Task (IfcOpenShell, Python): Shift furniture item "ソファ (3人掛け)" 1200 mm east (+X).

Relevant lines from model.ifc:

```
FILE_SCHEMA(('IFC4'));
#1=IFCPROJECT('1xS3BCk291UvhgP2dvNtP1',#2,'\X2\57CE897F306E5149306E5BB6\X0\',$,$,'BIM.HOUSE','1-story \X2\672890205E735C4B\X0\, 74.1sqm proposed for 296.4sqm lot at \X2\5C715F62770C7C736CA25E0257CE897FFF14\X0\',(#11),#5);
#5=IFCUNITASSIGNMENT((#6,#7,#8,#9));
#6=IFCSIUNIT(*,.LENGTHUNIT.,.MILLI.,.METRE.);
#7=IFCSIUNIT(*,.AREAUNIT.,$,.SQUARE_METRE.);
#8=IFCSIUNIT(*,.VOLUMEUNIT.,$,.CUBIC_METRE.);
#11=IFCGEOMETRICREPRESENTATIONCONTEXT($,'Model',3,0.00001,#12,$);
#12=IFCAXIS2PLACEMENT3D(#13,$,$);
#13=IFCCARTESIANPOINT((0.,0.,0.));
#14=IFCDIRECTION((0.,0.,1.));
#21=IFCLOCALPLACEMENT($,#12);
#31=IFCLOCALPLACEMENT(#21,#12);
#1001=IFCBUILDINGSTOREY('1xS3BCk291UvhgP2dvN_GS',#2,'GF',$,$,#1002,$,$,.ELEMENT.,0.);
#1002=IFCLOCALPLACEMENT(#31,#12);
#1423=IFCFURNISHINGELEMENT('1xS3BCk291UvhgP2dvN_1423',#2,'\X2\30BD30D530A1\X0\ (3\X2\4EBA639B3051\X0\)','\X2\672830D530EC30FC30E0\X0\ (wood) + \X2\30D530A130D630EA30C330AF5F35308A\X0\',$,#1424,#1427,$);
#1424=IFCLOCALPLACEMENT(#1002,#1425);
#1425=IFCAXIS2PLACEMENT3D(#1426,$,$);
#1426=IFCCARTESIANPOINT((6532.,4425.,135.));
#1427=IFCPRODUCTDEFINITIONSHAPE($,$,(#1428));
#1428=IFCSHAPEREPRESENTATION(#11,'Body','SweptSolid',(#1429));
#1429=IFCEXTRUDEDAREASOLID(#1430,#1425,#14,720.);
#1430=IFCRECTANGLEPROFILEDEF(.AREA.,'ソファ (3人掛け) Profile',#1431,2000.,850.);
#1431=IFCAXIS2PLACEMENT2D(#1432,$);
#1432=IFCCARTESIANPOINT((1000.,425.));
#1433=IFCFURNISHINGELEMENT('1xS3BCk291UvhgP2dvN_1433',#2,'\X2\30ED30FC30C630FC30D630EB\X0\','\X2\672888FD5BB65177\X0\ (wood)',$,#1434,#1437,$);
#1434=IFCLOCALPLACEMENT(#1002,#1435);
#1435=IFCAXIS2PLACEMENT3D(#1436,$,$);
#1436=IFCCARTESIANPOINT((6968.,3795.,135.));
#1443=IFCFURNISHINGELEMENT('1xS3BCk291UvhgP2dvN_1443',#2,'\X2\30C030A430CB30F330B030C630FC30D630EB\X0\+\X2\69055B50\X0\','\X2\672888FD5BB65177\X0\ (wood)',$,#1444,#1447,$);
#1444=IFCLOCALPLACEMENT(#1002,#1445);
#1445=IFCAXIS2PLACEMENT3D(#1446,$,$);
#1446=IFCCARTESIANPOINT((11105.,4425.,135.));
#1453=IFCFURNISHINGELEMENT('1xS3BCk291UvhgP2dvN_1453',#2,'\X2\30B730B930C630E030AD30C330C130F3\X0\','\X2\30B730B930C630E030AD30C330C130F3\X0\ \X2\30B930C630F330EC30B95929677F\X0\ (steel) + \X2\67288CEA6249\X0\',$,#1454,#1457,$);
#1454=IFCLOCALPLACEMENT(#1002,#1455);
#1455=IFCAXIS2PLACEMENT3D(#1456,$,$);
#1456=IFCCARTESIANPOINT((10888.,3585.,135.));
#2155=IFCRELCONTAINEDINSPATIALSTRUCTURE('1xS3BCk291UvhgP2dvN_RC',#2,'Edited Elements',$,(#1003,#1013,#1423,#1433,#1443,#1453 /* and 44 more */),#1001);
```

```python
import ifcopenshell
import ifcopenshell.api.geometry
import ifcopenshell.util.placement

model = ifcopenshell.open("model.ifc")

item = model.by_guid("1xS3BCk291UvhgP2dvN_1423")
matrix = ifcopenshell.util.placement.get_local_placement(item.ObjectPlacement)
matrix[0, 3] += 1200.0
ifcopenshell.api.geometry.edit_object_placement(model, product=item, matrix=matrix, is_si=False)

print(ifcopenshell.util.placement.get_local_placement(item.ObjectPlacement).round(3) + 0.0)

model.write("model-out.ifc")
```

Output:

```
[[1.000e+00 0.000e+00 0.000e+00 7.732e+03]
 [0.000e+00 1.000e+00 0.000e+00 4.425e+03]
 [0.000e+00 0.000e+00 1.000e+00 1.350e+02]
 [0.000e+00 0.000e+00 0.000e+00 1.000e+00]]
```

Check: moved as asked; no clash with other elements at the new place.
